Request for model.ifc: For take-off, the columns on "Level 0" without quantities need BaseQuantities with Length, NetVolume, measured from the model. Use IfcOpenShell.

First a look at what the model holds.

```python
import ifcopenshell
import ifcopenshell.util.element
import ifcopenshell.util.unit

model = ifcopenshell.open("model.ifc")
print(model.schema)
for unit_type in ("LENGTHUNIT", "AREAUNIT", "VOLUMEUNIT"):
    print(unit_type, ifcopenshell.util.unit.calculate_unit_scale(model, unit_type))
storey = next(s for s in model.by_type("IfcBuildingStorey") if s.Name == "Level 0")
columns = [e for e in ifcopenshell.util.element.get_decomposition(storey) if e.is_a("IfcColumn")]
for e in sorted(columns, key=lambda e: e.id()):
    print(e.id(), e.is_a(), e.Name, list(ifcopenshell.util.element.get_psets(e, qtos_only=True)), sep=" | ")
```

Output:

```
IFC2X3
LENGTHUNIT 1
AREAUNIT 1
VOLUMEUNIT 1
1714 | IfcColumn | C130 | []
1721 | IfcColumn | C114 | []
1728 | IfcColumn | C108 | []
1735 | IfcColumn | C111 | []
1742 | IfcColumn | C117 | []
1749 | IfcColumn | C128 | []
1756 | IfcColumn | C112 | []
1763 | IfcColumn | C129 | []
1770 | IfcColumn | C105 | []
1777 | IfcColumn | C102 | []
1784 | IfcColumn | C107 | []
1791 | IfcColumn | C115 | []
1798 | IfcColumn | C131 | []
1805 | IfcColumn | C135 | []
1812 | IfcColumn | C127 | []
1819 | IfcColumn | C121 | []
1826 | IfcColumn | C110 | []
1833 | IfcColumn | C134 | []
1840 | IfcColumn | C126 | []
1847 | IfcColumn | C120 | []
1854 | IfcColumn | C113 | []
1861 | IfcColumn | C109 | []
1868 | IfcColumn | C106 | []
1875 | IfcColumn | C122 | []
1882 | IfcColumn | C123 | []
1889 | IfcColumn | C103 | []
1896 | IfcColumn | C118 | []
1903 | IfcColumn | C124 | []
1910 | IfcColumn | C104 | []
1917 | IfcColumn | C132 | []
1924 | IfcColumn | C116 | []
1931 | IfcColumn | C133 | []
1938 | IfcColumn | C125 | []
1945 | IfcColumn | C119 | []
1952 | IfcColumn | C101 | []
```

```python
import ifcopenshell
import ifcopenshell.api.pset
import ifcopenshell.geom
import ifcopenshell.util.element
import ifcopenshell.util.shape
import ifcopenshell.util.unit

model = ifcopenshell.open("model.ifc")
unit_scale = ifcopenshell.util.unit.calculate_unit_scale(model)
volume_scale = ifcopenshell.util.unit.calculate_unit_scale(model, "VOLUMEUNIT")
settings = ifcopenshell.geom.settings()

storey = next(s for s in model.by_type("IfcBuildingStorey") if s.Name == "Level 0")
columns = [e for e in ifcopenshell.util.element.get_decomposition(storey) if e.is_a("IfcColumn")]

for e in sorted(columns, key=lambda e: e.id()):
    if ifcopenshell.util.element.get_psets(e, qtos_only=True, should_inherit=False):
        continue
    # Geometry comes back in metres, in the element's own axes.
    shape = ifcopenshell.geom.create_shape(settings, e)
    values = {
        "Length": ifcopenshell.util.shape.get_z(shape.geometry) / unit_scale,
        "NetVolume": ifcopenshell.util.shape.get_volume(shape.geometry) / volume_scale,
    }
    qto = ifcopenshell.api.pset.add_qto(model, product=e, name="BaseQuantities")
    ifcopenshell.api.pset.edit_qto(model, qto=qto, properties=values)
    print(e.id(), {k: round(v, 3) for k, v in values.items()})

model.write("model_v2.ifc")
```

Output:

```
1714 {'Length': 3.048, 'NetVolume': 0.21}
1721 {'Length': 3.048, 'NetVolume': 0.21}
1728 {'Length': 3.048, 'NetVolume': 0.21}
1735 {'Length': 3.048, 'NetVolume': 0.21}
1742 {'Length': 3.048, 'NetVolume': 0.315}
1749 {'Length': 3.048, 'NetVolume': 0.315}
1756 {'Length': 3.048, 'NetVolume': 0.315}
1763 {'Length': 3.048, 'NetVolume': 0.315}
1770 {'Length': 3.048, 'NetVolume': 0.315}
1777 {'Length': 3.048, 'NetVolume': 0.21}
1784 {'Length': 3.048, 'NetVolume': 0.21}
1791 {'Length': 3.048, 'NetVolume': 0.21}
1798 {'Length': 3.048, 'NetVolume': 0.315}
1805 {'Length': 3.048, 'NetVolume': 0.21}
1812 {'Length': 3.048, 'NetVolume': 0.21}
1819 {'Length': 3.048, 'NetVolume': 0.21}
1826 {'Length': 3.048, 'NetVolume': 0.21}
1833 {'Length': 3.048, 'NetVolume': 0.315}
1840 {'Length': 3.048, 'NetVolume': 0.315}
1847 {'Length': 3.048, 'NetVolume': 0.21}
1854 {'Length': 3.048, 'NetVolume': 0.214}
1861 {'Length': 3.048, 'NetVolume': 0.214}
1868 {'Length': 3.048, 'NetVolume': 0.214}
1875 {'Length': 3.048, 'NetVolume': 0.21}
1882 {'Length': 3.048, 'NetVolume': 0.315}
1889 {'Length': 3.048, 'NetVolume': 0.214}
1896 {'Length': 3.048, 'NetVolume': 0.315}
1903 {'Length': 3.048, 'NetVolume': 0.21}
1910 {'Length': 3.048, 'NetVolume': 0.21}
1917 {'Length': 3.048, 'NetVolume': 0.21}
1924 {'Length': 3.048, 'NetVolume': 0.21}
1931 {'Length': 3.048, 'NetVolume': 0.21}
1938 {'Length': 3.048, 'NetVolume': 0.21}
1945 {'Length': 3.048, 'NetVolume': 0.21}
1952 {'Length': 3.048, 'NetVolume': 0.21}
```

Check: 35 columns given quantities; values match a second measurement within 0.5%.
